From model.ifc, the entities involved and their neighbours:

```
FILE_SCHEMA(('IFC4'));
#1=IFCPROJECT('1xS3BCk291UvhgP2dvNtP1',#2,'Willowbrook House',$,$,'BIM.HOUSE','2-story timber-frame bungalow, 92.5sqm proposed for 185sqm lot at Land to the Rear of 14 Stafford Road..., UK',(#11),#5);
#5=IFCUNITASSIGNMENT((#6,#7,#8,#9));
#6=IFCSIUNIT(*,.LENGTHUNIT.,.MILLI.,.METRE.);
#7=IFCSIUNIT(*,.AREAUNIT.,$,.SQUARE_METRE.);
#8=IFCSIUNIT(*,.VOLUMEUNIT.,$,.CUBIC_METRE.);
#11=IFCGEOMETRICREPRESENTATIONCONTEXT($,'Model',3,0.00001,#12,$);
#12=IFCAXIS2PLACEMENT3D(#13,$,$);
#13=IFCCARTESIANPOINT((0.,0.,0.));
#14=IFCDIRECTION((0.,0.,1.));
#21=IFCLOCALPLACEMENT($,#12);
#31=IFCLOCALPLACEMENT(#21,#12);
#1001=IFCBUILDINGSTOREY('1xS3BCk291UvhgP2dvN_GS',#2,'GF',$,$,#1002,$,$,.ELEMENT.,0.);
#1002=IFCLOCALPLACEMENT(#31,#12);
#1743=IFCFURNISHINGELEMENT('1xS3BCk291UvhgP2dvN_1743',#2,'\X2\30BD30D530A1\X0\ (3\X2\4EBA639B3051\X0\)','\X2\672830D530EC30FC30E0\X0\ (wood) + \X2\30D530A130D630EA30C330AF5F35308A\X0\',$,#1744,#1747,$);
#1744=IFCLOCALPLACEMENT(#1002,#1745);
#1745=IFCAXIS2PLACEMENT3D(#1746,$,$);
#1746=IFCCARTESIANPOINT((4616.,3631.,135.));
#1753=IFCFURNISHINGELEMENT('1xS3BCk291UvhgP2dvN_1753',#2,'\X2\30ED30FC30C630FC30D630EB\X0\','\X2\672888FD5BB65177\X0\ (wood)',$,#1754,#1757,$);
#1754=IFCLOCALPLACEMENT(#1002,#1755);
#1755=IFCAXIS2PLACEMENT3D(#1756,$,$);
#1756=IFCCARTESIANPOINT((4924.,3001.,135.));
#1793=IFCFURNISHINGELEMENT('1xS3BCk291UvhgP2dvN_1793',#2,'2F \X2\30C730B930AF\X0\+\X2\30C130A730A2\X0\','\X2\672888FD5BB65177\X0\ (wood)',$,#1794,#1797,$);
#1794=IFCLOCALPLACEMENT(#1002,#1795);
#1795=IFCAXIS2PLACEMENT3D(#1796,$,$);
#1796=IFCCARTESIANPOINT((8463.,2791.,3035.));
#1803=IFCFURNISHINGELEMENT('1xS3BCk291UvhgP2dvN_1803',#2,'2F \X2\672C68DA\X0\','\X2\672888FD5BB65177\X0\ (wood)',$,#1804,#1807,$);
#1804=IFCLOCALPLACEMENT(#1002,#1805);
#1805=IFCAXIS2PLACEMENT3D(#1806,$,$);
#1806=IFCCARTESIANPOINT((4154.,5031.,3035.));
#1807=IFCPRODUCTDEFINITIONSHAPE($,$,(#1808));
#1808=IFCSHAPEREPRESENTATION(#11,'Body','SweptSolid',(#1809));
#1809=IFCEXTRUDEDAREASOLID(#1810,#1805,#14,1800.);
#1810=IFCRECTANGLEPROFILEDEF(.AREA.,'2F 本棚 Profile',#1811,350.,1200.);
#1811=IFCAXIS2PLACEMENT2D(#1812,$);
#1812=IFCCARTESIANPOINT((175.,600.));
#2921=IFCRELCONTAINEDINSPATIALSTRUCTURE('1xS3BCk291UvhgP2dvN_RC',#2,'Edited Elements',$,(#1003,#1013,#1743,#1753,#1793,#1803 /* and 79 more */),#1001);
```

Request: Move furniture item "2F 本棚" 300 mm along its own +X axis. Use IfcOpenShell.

```python
import ifcopenshell
import ifcopenshell.api.geometry
import ifcopenshell.util.placement

model = ifcopenshell.open("model.ifc")

item = model.by_guid("1xS3BCk291UvhgP2dvN_1803")
matrix = ifcopenshell.util.placement.get_local_placement(item.ObjectPlacement)
matrix[:3, 3] += matrix[:3, 0] * 300.0
ifcopenshell.api.geometry.edit_object_placement(model, product=item, matrix=matrix, is_si=False)

print(ifcopenshell.util.placement.get_local_placement(item.ObjectPlacement).round(3) + 0.0)

model.write("model_edited.ifc")
```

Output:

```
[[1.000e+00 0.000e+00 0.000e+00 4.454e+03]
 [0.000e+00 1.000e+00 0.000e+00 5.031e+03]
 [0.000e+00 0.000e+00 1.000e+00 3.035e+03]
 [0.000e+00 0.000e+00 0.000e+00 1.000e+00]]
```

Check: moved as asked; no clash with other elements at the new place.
